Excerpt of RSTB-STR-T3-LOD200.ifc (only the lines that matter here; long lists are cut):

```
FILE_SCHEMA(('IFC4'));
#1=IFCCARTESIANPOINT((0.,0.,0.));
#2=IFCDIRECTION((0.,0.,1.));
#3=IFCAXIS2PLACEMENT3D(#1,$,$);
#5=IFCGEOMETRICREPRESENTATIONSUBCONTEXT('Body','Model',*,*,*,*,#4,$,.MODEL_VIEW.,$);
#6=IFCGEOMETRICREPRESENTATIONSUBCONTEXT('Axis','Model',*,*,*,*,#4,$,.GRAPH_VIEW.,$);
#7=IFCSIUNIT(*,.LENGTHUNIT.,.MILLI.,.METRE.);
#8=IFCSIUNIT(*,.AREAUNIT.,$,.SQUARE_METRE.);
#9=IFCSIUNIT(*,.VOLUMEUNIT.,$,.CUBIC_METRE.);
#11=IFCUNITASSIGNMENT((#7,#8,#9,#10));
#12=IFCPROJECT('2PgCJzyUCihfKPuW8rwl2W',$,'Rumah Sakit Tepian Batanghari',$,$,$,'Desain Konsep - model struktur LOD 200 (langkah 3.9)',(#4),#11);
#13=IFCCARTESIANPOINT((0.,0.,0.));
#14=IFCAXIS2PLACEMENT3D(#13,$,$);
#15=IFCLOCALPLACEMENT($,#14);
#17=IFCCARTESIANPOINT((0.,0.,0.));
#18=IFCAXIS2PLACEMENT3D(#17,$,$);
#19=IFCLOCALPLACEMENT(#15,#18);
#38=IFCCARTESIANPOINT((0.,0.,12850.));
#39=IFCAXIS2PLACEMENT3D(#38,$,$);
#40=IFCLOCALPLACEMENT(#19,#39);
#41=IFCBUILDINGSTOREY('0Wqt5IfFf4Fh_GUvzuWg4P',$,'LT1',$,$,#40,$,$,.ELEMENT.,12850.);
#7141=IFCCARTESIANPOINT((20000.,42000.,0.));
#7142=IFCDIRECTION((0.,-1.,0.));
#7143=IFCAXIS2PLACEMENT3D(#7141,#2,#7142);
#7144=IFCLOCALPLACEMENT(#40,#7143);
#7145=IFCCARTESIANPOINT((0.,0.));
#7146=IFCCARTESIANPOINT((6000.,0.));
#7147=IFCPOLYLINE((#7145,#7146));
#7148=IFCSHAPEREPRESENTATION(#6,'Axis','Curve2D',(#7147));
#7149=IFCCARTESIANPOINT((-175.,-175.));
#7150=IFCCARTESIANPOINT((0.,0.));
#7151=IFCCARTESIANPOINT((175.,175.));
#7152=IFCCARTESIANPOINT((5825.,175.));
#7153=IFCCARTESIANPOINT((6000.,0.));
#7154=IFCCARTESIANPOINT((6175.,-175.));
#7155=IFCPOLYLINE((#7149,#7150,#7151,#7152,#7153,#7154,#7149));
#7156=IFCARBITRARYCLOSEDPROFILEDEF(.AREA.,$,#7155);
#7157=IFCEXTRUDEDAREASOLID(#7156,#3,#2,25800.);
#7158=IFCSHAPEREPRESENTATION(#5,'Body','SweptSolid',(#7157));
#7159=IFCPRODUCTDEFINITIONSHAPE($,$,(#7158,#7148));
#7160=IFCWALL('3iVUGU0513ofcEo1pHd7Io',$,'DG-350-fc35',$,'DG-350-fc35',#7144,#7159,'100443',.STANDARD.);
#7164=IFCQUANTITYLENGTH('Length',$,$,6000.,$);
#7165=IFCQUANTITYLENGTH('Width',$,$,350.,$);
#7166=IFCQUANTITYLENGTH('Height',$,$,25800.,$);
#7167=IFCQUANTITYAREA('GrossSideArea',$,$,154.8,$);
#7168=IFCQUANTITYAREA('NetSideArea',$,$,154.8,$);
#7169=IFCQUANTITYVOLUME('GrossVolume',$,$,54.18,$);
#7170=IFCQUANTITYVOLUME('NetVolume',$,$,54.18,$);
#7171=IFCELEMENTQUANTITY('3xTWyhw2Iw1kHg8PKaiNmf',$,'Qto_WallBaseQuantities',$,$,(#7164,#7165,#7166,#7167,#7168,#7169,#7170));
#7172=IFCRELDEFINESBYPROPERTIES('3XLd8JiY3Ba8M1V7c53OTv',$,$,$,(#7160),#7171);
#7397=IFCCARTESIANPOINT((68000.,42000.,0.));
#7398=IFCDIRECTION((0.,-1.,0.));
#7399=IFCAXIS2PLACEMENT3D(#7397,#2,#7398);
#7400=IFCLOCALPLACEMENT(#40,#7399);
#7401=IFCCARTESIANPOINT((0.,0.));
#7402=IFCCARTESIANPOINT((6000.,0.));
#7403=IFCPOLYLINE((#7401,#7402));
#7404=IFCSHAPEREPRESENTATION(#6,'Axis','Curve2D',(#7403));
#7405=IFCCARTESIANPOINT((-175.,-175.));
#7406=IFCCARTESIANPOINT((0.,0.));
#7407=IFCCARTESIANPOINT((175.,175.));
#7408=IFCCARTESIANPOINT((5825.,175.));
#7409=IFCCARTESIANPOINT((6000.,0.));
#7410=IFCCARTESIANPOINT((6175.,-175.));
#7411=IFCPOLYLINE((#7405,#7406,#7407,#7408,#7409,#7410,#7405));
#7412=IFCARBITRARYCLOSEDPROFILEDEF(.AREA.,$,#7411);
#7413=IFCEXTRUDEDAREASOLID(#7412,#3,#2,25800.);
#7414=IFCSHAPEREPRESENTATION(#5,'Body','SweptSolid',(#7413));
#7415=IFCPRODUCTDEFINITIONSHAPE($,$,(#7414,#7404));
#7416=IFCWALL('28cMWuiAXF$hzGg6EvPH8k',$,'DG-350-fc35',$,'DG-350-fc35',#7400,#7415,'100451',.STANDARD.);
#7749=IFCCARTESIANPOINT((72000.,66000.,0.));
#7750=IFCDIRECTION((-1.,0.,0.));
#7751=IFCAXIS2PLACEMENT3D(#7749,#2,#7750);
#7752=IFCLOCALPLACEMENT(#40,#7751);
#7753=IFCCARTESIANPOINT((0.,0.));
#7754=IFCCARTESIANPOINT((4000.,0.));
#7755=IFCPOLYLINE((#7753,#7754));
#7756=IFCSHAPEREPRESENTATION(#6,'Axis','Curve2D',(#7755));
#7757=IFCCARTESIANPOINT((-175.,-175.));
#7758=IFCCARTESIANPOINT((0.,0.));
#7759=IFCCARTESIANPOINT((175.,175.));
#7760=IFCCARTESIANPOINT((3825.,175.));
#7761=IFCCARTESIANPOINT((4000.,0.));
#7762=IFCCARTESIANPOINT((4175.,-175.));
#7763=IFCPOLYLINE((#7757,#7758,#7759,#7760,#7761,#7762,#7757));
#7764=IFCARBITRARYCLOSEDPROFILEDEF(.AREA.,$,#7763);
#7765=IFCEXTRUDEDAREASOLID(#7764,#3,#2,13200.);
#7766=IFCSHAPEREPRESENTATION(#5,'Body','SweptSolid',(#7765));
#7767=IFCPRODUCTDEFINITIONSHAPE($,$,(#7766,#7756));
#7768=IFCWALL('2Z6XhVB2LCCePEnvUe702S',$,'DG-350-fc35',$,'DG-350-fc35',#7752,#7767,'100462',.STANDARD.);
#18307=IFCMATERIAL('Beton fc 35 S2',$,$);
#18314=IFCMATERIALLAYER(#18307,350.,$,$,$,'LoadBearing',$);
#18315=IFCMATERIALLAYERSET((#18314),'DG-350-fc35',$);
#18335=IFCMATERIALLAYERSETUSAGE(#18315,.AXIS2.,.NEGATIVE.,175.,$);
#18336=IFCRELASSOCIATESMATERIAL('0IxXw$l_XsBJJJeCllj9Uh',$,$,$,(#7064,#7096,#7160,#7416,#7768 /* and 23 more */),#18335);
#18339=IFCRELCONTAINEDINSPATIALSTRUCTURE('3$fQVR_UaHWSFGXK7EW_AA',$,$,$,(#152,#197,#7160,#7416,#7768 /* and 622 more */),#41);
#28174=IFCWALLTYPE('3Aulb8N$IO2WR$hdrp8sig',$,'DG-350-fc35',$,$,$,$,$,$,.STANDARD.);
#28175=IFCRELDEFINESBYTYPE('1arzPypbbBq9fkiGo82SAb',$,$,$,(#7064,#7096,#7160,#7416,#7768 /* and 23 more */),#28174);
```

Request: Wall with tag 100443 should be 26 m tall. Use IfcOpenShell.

```python
import ifcopenshell
import ifcopenshell.api.pset
import ifcopenshell.geom
import ifcopenshell.util.element
import ifcopenshell.util.representation
import ifcopenshell.util.shape
import ifcopenshell.util.unit

model = ifcopenshell.open("RSTB-STR-T3-LOD200.ifc")
unit_scale = ifcopenshell.util.unit.calculate_unit_scale(model)
area_scale = ifcopenshell.util.unit.calculate_unit_scale(model, "AREAUNIT")
volume_scale = ifcopenshell.util.unit.calculate_unit_scale(model, "VOLUMEUNIT")
settings = ifcopenshell.geom.settings()


def volume(element):
    """Net volume in cubic metres, openings subtracted."""
    shape = ifcopenshell.geom.create_shape(settings, element)
    return ifcopenshell.util.shape.get_volume(shape.geometry)


wall = model.by_guid("3iVUGU0513ofcEo1pHd7Io")
before = volume(wall)

body = ifcopenshell.util.representation.get_representation(wall, "Model", "Body")
solid = body.Items[0]
old_height = solid.Depth
solid.Depth = 26 / unit_scale
after = volume(wall)
thickness = 0.35  # wall thickness in metres

# Update the stored height, areas and volumes.
qto = model.by_id(ifcopenshell.util.element.get_pset(wall, "Qto_WallBaseQuantities", should_inherit=False)["id"])
ifcopenshell.api.pset.edit_qto(model, qto=qto, properties={
    "Height": solid.Depth,
    "GrossSideArea": ifcopenshell.util.element.get_pset(wall, "Qto_WallBaseQuantities", "GrossSideArea") * solid.Depth / old_height,
    "NetSideArea": after / thickness / area_scale,
    "GrossVolume": ifcopenshell.util.element.get_pset(wall, "Qto_WallBaseQuantities", "GrossVolume") * solid.Depth / old_height,
    "NetVolume": after / volume_scale,
})

print(f"height {old_height:g} -> {solid.Depth:g}, volume {before:.3f} -> {after:.3f} m3")

model.write("RSTB-STR-T3-LOD200_v2.ifc")
```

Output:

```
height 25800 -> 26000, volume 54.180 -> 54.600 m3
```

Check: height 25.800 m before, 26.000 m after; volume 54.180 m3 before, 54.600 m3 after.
